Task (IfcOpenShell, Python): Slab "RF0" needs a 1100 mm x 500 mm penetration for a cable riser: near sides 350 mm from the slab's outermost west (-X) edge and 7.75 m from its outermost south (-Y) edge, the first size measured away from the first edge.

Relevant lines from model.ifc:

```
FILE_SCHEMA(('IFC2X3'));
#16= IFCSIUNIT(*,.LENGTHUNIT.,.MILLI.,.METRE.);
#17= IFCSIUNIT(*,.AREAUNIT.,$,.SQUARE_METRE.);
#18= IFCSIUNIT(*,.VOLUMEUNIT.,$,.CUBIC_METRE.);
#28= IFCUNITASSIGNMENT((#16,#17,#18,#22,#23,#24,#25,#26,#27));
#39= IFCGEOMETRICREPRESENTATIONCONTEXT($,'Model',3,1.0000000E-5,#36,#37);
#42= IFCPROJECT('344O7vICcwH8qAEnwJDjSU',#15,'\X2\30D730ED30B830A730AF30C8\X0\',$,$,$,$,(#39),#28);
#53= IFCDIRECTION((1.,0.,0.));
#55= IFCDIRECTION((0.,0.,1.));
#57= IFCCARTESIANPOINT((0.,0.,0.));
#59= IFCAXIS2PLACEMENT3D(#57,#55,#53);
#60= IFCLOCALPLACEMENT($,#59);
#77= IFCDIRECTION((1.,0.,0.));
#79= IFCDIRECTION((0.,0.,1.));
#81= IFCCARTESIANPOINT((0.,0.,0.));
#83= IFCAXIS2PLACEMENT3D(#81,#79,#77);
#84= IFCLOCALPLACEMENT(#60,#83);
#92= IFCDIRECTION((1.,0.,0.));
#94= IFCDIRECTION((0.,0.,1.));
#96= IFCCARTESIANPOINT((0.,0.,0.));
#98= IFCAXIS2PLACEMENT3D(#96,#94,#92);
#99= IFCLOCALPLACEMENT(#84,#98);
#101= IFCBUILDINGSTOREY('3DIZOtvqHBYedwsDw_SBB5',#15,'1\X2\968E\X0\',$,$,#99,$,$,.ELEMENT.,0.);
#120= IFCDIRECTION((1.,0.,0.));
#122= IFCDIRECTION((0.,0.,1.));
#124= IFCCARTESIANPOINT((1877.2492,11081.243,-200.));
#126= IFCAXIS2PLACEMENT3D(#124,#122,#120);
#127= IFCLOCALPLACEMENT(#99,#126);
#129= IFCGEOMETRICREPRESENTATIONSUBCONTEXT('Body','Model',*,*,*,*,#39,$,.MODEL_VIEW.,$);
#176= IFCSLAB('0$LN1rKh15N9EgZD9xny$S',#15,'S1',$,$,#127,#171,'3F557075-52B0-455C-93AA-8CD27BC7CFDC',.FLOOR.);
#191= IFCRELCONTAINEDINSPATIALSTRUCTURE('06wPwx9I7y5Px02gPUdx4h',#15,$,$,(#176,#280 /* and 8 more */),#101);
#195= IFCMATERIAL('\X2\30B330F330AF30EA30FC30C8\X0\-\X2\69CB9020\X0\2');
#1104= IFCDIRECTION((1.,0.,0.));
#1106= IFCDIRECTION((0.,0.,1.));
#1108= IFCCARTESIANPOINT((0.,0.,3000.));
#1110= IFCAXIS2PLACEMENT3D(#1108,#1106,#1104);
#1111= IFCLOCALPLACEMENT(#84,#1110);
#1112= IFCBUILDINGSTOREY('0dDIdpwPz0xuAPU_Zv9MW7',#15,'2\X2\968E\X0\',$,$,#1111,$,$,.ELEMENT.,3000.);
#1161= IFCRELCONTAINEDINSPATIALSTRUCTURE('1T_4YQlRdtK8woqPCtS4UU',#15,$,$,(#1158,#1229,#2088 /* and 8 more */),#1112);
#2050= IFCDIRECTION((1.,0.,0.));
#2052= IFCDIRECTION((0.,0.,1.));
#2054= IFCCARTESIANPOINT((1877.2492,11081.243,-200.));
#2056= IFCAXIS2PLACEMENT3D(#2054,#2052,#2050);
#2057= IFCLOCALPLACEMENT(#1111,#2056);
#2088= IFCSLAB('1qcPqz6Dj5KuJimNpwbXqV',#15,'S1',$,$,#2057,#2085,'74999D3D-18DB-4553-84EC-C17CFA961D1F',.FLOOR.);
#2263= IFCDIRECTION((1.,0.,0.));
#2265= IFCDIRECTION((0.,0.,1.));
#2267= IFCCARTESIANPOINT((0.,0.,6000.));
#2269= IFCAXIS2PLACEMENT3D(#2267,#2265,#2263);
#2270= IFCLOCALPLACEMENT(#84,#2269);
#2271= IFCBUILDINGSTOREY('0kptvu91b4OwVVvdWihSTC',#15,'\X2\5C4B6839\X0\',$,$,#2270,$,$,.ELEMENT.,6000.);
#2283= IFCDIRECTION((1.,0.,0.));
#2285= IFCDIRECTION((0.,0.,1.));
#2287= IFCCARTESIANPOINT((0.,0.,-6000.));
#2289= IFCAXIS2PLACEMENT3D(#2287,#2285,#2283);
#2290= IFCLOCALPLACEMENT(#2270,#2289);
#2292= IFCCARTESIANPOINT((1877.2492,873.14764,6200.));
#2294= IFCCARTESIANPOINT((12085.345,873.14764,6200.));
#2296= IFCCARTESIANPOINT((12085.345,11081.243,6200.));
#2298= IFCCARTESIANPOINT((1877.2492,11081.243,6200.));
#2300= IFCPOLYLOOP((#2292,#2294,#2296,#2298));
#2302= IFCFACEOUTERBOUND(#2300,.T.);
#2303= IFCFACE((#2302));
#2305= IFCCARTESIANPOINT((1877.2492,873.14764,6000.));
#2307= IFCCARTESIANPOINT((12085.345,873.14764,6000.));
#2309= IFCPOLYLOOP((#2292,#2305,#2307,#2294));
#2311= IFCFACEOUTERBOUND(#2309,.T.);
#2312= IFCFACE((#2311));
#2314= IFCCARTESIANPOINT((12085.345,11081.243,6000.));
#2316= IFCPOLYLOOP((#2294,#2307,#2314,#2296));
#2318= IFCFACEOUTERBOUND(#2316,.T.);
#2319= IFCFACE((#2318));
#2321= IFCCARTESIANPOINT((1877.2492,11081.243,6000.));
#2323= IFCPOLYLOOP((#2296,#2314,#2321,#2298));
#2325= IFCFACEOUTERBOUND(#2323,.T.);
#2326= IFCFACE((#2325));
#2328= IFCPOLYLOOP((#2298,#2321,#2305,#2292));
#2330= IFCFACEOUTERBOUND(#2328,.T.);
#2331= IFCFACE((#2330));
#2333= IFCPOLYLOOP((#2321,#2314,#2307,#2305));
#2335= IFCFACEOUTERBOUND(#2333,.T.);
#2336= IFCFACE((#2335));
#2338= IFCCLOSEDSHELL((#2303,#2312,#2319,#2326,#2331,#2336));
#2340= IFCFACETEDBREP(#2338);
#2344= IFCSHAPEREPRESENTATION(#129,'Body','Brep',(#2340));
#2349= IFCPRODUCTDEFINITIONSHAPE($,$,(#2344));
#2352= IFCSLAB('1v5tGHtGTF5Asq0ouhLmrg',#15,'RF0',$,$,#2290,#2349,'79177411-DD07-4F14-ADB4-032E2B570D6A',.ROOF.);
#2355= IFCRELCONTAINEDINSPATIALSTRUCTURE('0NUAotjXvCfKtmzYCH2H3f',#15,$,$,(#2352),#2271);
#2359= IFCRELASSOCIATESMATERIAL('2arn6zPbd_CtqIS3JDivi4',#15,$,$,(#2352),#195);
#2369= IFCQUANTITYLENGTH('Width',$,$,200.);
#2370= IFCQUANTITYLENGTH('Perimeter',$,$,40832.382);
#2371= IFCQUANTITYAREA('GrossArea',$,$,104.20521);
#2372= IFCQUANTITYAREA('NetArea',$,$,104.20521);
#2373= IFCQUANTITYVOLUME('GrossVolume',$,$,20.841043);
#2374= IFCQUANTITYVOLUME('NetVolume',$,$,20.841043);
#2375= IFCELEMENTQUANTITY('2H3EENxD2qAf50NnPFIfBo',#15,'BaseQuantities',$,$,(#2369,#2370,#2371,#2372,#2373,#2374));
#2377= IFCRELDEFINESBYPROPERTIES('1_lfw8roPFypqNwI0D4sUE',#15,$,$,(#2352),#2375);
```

```python
import numpy as np
import ifcopenshell
import ifcopenshell.api.feature
import ifcopenshell.api.geometry
import ifcopenshell.api.pset
import ifcopenshell.api.root
import ifcopenshell.geom
import ifcopenshell.util.element
import ifcopenshell.util.placement
import ifcopenshell.util.representation
import ifcopenshell.util.shape
import ifcopenshell.util.unit

model = ifcopenshell.open("model.ifc")
unit_scale = ifcopenshell.util.unit.calculate_unit_scale(model)
area_scale = ifcopenshell.util.unit.calculate_unit_scale(model, "AREAUNIT")
volume_scale = ifcopenshell.util.unit.calculate_unit_scale(model, "VOLUMEUNIT")
settings = ifcopenshell.geom.settings()


def volume(element):
    """Net volume in cubic metres, openings subtracted."""
    shape = ifcopenshell.geom.create_shape(settings, element)
    return ifcopenshell.util.shape.get_volume(shape.geometry)


slab = model.by_guid("1v5tGHtGTF5Asq0ouhLmrg")
before = volume(slab)

# Extent in the slab's own axes, in metres. The edges named are its -X and -Y sides.
slab_shape = ifcopenshell.geom.create_shape(settings, slab)
vertices = ifcopenshell.util.shape.get_vertices(slab_shape.geometry)
x_min, y_min, bottom = vertices.min(axis=0)
top = vertices[:, 2].max()

opening = ifcopenshell.api.root.create_entity(model, ifc_class="IfcOpeningElement", name="Cable riser opening")
context = ifcopenshell.util.representation.get_context(model, "Model", "Body", "MODEL_VIEW")
width, depth = 1.1, 0.5
outline = [(0.0, 0.0), (width, 0.0), (width, depth), (0.0, depth), (0.0, 0.0)]
# Overshoot both faces by 50 mm so the cut is clean.
shape = ifcopenshell.api.geometry.add_slab_representation(
    model, context=context, depth=top - bottom + 0.1, polyline=outline
)
ifcopenshell.api.geometry.assign_representation(model, product=opening, representation=shape)

matrix = ifcopenshell.util.placement.get_local_placement(slab.ObjectPlacement)
matrix[:, 3] = matrix @ np.append(np.array([x_min + 0.35, y_min + 7.75, bottom - 0.05]) / unit_scale, 1.0)
ifcopenshell.api.geometry.edit_object_placement(model, product=opening, matrix=matrix, is_si=False)
ifcopenshell.api.feature.add_feature(model, feature=opening, element=slab)

after = volume(slab)

# Update the slab's stored quantities.
qto = model.by_id(ifcopenshell.util.element.get_pset(slab, "BaseQuantities", should_inherit=False)["id"])
ifcopenshell.api.pset.edit_qto(model, qto=qto, properties={
    "NetArea": after / (top - bottom) / area_scale,
    "NetVolume": after / volume_scale,
})

print(f"slab volume {before:.3f} -> {after:.3f} m3")

model.write("model_rev.ifc")
```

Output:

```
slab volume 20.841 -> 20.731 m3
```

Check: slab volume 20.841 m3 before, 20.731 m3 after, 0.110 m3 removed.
